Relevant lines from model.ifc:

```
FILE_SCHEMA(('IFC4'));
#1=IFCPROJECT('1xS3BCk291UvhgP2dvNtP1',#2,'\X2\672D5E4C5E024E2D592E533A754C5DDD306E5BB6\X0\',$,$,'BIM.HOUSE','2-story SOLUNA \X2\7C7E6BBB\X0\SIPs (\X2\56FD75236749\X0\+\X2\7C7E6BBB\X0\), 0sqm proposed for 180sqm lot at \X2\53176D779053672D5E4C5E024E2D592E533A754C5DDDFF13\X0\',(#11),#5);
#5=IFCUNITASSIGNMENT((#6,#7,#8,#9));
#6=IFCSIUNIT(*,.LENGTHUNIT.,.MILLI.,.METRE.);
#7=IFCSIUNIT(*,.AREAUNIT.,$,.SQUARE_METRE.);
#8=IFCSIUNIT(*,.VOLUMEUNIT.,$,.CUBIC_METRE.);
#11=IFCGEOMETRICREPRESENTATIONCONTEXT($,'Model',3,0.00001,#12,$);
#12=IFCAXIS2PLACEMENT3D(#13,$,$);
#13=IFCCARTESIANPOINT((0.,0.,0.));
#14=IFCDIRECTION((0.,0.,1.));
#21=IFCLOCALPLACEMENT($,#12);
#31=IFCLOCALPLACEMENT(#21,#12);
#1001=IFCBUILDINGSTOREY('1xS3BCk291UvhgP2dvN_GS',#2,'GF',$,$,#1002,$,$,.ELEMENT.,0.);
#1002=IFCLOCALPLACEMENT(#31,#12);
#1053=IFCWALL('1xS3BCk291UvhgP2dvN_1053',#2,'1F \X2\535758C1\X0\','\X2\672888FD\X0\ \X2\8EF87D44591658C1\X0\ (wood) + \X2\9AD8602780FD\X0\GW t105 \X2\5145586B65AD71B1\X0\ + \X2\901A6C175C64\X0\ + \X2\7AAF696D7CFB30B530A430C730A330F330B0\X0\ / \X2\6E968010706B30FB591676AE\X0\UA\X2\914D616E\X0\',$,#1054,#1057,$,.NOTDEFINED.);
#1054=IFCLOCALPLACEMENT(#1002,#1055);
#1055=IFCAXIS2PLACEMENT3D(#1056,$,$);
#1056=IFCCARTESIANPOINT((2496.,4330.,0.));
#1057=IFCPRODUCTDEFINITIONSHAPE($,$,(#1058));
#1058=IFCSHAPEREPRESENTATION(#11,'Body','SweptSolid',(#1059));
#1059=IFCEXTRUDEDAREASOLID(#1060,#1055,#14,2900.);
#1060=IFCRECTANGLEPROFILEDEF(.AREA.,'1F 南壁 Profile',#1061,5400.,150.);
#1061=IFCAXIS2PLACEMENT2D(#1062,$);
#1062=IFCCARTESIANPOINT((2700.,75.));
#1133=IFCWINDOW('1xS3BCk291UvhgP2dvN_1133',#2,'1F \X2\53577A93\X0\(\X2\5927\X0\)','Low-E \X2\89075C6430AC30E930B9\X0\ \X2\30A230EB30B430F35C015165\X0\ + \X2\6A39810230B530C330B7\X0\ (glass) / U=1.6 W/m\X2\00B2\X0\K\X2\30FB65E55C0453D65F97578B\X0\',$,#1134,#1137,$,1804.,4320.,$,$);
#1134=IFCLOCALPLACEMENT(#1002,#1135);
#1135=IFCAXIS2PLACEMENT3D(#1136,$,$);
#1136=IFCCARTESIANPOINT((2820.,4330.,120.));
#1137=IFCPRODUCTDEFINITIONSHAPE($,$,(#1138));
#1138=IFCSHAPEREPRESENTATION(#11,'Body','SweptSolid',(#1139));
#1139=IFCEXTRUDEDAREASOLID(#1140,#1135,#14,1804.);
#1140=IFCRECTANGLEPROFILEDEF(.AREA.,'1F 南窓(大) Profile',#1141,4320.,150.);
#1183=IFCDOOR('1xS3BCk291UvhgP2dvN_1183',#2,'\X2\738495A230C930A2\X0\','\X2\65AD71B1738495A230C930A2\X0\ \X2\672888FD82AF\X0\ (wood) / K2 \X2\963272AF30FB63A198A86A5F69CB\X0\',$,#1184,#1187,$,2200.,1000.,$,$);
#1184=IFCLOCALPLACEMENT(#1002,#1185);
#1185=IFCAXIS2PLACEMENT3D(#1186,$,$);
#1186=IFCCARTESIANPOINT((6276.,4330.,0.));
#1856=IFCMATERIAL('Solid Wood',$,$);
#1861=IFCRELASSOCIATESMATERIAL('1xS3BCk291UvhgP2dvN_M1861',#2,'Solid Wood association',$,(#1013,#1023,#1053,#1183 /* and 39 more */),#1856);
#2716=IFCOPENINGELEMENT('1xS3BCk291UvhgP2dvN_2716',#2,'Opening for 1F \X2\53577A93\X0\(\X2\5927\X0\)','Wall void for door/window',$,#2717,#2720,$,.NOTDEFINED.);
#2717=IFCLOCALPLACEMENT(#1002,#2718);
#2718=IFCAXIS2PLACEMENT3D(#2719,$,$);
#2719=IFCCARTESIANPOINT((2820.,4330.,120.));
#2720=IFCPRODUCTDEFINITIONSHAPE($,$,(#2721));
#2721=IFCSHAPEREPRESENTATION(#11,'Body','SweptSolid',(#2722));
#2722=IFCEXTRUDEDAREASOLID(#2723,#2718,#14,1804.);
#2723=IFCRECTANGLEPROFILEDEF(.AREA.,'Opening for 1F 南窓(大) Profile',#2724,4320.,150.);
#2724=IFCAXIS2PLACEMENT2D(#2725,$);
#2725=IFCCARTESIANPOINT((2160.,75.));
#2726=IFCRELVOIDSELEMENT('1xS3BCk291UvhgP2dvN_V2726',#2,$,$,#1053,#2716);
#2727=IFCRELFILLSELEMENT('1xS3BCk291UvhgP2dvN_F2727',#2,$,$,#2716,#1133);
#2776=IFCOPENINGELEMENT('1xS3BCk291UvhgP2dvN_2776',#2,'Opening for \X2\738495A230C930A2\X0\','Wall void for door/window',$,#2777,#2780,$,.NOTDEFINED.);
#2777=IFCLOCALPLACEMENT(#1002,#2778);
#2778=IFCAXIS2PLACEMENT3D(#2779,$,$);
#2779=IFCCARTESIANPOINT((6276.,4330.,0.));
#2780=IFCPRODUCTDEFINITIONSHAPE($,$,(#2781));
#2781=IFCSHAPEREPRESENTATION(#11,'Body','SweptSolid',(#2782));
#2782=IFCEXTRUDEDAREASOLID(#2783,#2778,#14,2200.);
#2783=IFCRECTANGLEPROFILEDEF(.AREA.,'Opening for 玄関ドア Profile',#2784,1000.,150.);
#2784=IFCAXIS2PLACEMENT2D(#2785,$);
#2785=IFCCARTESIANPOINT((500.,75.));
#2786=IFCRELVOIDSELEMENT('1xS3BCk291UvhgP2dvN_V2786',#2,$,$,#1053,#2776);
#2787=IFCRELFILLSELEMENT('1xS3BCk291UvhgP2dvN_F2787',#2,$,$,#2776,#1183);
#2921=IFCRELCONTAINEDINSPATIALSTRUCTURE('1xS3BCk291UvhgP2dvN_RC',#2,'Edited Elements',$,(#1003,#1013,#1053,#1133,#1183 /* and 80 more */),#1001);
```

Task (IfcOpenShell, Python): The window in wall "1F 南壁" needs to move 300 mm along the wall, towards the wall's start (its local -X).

```python
import ifcopenshell
import ifcopenshell.api.geometry
import ifcopenshell.util.placement
import ifcopenshell.util.unit

model = ifcopenshell.open("model.ifc")
unit_scale = ifcopenshell.util.unit.calculate_unit_scale(model)

window = model.by_guid("1xS3BCk291UvhgP2dvN_1133")
opening = window.FillsVoids[0].RelatingOpeningElement
wall = opening.VoidsElements[0].RelatingBuildingElement

wall_matrix = ifcopenshell.util.placement.get_local_placement(wall.ObjectPlacement)
shift = wall_matrix[:3, 0] * -0.3 / unit_scale
before = ifcopenshell.util.placement.get_local_placement(window.ObjectPlacement)[:3, 3].copy()

# The window is not placed relative to its opening, so move both.
for product in (opening, window):
    matrix = ifcopenshell.util.placement.get_local_placement(product.ObjectPlacement)
    matrix[:3, 3] += shift
    ifcopenshell.api.geometry.edit_object_placement(model, product=product, matrix=matrix, is_si=False)

after = ifcopenshell.util.placement.get_local_placement(window.ObjectPlacement)[:3, 3]
print("window moved by", (after - before).round(3) + 0.0)

model.write("model-out.ifc")
```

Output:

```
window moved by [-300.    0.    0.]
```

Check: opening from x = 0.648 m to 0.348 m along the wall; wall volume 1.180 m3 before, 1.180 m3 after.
